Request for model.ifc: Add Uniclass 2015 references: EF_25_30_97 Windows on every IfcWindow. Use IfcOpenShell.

First a look at what the model holds.

```python
import ifcopenshell

model = ifcopenshell.open("model.ifc")
print(model.schema)
print("classifications:", [c.Name for c in model.by_type("IfcClassification")])
for ifc_class in ("IfcDoor", "IfcRoof", "IfcStair", "IfcWall", "IfcWindow"):
    print(ifc_class, len(model.by_type(ifc_class)))
```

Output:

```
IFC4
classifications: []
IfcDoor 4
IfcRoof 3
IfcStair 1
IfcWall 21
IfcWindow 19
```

```python
import ifcopenshell
import ifcopenshell.api.classification

model = ifcopenshell.open("model.ifc")

system = ifcopenshell.api.classification.add_classification(model, classification="Uniclass 2015")

codes = {
    "IfcWindow": ("EF_25_30_97", "Windows"),
}
for ifc_class, (code, name) in codes.items():
    products = model.by_type(ifc_class)
    ifcopenshell.api.classification.add_reference(
        model, products=products, classification=system, identification=code, name=name
    )
    print(code, len(products))

model.write("model-out.ifc")
```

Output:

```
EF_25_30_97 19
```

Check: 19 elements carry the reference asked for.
